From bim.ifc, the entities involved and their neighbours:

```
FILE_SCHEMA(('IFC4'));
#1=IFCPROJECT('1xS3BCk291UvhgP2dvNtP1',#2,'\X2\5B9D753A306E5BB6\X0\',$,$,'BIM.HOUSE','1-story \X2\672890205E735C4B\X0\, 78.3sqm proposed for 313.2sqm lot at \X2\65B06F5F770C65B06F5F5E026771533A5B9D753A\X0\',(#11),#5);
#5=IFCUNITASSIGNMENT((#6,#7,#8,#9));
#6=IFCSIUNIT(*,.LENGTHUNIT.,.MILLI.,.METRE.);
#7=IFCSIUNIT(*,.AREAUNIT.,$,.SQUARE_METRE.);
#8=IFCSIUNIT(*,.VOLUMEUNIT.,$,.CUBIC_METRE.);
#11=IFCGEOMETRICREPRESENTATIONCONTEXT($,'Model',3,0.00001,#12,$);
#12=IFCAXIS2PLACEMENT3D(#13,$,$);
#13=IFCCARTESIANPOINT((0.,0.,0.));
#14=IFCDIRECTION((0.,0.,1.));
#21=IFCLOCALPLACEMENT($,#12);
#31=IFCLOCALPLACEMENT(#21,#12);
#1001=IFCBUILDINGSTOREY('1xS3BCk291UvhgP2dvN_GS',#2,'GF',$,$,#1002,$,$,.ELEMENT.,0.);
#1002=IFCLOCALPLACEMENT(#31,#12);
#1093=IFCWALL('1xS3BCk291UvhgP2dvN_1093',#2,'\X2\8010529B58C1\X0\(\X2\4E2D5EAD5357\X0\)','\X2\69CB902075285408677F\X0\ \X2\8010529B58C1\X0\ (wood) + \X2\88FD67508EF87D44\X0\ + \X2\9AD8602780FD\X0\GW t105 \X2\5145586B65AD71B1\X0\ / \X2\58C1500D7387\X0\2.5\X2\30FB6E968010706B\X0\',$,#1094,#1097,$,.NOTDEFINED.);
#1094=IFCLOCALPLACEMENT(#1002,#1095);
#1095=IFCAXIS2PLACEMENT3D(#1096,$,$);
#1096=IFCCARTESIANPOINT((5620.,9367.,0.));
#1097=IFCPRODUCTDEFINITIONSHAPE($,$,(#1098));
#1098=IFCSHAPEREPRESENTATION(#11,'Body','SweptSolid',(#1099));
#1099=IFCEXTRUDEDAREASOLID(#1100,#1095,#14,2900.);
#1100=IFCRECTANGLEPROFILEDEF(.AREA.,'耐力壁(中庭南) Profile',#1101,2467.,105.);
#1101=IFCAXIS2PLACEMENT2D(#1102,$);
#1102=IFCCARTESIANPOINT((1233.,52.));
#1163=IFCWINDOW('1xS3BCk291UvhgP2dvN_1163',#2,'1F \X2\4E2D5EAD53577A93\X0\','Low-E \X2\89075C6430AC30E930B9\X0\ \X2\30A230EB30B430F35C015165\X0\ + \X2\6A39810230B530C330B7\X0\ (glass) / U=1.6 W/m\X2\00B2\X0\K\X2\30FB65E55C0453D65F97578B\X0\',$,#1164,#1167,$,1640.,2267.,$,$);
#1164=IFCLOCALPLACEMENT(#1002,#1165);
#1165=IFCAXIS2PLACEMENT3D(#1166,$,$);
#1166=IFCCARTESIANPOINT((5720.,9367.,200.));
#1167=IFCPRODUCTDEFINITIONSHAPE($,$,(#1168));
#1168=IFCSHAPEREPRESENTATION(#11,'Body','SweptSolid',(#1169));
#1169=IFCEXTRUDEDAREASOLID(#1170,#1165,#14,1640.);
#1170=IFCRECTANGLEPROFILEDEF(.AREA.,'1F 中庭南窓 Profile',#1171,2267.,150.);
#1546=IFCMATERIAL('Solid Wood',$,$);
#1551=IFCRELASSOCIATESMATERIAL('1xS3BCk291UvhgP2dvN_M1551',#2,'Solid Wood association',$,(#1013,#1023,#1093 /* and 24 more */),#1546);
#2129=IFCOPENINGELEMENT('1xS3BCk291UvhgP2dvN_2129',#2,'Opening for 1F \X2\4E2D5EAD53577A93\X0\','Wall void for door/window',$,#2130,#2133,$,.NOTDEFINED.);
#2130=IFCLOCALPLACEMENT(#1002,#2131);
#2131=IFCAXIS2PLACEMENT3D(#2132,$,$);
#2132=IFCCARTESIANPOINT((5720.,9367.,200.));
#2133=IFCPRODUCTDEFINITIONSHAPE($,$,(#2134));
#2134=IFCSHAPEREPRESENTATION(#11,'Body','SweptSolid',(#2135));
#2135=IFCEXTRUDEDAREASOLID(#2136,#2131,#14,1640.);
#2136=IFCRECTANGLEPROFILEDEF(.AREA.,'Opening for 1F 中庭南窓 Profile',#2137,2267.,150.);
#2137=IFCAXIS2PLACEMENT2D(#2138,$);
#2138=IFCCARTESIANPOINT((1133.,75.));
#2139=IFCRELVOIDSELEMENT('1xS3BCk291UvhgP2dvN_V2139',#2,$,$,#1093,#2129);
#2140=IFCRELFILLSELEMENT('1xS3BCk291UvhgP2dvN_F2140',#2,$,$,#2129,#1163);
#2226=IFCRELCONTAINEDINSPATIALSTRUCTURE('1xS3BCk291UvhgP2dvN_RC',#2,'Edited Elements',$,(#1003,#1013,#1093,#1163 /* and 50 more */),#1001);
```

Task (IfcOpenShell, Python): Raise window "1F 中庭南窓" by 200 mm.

```python
import numpy as np
import ifcopenshell
import ifcopenshell.api.geometry
import ifcopenshell.util.placement
import ifcopenshell.util.unit

model = ifcopenshell.open("bim.ifc")
unit_scale = ifcopenshell.util.unit.calculate_unit_scale(model)

window = model.by_id(1163)
opening = window.FillsVoids[0].RelatingOpeningElement
dz = 200.0

shift = np.array([0.0, 0.0, dz])
# The window is not placed relative to its opening, so move both.
for product in (opening, window):
    matrix = ifcopenshell.util.placement.get_local_placement(product.ObjectPlacement)
    matrix[:3, 3] += shift
    ifcopenshell.api.geometry.edit_object_placement(model, product=product, matrix=matrix, is_si=False)

print(f"moved by {dz * unit_scale:+.3f} m")

model.write("bim_updated.ifc")
```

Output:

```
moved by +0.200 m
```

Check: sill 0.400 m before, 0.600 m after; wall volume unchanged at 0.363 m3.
